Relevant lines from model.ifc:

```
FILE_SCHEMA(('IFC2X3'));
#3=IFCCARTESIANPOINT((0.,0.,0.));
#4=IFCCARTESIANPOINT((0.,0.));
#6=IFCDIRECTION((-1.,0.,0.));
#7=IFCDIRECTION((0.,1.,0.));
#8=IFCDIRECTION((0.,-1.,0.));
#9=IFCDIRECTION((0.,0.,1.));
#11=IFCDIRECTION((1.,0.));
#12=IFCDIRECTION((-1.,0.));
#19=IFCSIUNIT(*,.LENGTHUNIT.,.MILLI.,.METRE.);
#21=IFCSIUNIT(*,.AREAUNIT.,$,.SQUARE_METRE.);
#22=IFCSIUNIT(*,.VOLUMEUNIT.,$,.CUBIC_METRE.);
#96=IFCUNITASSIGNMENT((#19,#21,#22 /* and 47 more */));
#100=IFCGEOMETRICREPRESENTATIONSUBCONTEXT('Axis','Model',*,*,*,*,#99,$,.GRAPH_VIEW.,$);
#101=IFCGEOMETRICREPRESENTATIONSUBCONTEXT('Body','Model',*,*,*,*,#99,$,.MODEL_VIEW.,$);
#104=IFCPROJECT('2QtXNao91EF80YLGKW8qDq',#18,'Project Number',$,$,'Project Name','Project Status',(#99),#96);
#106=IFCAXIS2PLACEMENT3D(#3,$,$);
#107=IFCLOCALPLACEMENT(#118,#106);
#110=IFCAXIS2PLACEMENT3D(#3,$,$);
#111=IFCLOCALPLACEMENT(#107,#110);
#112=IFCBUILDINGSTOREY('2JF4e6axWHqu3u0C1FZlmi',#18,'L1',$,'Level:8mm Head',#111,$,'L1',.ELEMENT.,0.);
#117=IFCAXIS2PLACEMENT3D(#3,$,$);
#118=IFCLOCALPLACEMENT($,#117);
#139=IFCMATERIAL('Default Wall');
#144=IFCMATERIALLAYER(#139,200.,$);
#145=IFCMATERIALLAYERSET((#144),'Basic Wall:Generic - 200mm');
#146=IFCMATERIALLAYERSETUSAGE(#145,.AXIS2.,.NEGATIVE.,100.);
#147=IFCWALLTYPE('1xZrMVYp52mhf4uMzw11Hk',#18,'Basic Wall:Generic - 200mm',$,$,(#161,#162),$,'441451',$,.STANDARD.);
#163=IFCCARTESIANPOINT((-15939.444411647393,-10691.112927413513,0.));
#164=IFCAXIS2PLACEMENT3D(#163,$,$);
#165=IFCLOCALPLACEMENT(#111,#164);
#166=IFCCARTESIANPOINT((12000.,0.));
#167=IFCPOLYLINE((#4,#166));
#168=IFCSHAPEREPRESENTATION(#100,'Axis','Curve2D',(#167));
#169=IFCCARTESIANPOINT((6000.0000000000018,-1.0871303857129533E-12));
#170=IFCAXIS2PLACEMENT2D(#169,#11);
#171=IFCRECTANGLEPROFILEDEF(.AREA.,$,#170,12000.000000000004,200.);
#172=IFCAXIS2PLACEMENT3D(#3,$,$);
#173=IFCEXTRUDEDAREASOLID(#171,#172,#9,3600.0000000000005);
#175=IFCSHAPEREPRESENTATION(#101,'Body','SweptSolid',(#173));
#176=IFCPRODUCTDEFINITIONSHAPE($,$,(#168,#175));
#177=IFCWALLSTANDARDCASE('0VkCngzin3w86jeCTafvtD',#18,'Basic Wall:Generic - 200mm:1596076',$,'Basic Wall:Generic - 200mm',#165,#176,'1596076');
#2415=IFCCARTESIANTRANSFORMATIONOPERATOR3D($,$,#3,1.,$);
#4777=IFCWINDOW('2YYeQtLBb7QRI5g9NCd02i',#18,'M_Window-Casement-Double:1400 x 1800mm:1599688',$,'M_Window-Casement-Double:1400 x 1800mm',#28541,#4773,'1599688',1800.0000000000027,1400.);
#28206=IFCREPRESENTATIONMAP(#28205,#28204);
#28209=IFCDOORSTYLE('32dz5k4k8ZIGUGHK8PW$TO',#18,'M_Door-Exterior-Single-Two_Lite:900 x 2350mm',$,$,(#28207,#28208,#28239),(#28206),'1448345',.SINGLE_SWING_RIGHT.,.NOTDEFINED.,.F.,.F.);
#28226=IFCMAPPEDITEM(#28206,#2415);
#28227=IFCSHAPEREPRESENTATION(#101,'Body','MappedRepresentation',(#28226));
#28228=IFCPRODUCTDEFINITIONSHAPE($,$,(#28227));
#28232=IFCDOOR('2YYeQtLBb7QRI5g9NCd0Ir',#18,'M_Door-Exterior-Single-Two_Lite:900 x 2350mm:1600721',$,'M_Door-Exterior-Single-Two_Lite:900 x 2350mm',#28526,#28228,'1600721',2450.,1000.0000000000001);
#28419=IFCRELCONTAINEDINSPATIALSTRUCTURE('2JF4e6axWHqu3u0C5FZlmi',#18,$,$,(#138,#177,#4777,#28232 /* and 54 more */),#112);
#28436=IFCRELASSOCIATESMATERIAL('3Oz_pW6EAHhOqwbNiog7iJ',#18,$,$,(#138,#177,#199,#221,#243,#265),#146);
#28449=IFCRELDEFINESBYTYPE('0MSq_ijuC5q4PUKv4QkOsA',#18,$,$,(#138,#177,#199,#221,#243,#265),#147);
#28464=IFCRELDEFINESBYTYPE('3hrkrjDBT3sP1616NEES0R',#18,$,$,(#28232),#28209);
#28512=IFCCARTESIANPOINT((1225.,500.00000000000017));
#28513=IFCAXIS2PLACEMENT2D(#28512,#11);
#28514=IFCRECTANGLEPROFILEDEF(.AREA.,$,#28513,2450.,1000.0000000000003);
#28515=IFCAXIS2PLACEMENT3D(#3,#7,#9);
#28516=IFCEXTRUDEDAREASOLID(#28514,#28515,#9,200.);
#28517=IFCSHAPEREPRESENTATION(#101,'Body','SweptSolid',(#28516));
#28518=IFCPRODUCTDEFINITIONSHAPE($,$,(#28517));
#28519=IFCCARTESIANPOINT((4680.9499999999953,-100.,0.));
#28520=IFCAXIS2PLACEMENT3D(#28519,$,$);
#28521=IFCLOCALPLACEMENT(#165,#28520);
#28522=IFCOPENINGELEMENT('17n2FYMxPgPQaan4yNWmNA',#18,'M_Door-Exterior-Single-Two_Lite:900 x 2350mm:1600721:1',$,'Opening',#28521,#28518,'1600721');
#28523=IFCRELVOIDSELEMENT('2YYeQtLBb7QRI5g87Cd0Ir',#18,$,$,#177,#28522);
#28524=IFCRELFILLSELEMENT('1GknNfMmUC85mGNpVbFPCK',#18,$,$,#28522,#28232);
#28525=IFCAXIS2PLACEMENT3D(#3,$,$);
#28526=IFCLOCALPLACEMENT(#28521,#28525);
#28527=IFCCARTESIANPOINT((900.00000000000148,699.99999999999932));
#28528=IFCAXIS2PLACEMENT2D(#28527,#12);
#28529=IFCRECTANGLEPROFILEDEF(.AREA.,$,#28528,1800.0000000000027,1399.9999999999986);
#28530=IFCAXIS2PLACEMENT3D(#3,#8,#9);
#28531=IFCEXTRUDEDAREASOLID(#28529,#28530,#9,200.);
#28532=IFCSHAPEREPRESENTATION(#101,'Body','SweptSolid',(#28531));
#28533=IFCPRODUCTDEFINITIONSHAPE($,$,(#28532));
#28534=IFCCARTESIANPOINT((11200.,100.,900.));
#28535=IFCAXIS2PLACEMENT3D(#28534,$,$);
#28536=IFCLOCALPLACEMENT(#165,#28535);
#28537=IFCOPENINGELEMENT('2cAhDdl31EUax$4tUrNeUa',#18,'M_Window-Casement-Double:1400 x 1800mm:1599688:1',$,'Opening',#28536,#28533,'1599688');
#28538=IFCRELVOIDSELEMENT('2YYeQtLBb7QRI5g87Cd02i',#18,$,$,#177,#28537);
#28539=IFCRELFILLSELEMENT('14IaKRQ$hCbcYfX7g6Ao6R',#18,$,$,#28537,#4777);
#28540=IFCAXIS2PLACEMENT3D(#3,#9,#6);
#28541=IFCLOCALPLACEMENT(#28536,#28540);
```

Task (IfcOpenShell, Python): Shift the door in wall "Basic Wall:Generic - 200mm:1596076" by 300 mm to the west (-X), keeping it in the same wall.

```python
import ifcopenshell
import ifcopenshell.api.geometry
import ifcopenshell.util.placement
import ifcopenshell.util.unit

model = ifcopenshell.open("model.ifc")
unit_scale = ifcopenshell.util.unit.calculate_unit_scale(model)

door = model.by_guid("2YYeQtLBb7QRI5g9NCd0Ir")
opening = door.FillsVoids[0].RelatingOpeningElement
wall = opening.VoidsElements[0].RelatingBuildingElement

wall_matrix = ifcopenshell.util.placement.get_local_placement(wall.ObjectPlacement)
shift = wall_matrix[:3, 0] * -0.3 / unit_scale
before = ifcopenshell.util.placement.get_local_placement(door.ObjectPlacement)[:3, 3].copy()

# The door is placed relative to its opening, so it follows when the opening moves.
matrix = ifcopenshell.util.placement.get_local_placement(opening.ObjectPlacement)
matrix[:3, 3] += shift
ifcopenshell.api.geometry.edit_object_placement(
    model, product=opening, matrix=matrix, is_si=False, should_transform_children=True
)

after = ifcopenshell.util.placement.get_local_placement(door.ObjectPlacement)[:3, 3]
print("door moved by", (after - before).round(3) + 0.0)

model.write("model_edited.ifc")
```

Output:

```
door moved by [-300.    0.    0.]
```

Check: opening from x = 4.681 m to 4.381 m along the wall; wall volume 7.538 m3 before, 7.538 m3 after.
